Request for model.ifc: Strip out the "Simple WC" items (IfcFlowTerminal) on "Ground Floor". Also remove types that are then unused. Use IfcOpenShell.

First a look at what the model holds.

```python
import ifcopenshell
import ifcopenshell.util.element

model = ifcopenshell.open("model.ifc")
print(model.schema)
storey = next(s for s in model.by_type("IfcBuildingStorey") if s.Name == "Ground Floor")
terminals = [e for e in ifcopenshell.util.element.get_decomposition(storey) if e.is_a("IfcFlowTerminal")]
seen = {}
for e in terminals:
    element_type = ifcopenshell.util.element.get_type(e)
    name = element_type.Name if element_type not in (None, e) else None
    seen[name] = seen.get(name, 0) + 1
for name, count in sorted(seen.items(), key=str):
    print(count, "x", name)
```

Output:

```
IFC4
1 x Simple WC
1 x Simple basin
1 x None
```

```python
import ifcopenshell
import ifcopenshell.api.root
import ifcopenshell.util.element

model = ifcopenshell.open("model.ifc")

storey = next(s for s in model.by_type("IfcBuildingStorey") if s.Name == "Ground Floor")
terminals = [e for e in ifcopenshell.util.element.get_decomposition(storey) if e.is_a("IfcFlowTerminal")]
targets = [e for e in terminals if (t := ifcopenshell.util.element.get_type(e)) not in (None, e) and t.Name == "Simple WC"]
types = {ifcopenshell.util.element.get_type(e) for e in targets} - {None, *targets}

for e in targets:
    ifcopenshell.api.root.remove_product(model, product=e)
print(len(targets), "removed")

unused = [t for t in types if not ifcopenshell.util.element.get_types(t)]
for t in unused:
    ifcopenshell.api.root.remove_product(model, product=t)
print(len(unused), "unused types removed")

model.write("model_rev.ifc")
```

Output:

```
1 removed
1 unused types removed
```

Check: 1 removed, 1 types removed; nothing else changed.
